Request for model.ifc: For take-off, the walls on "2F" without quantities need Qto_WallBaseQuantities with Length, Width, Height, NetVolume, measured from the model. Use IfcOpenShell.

First a look at what the model holds.

```python
import ifcopenshell
import ifcopenshell.util.element
import ifcopenshell.util.unit

model = ifcopenshell.open("model.ifc")
print(model.schema)
for unit_type in ("LENGTHUNIT", "AREAUNIT", "VOLUMEUNIT"):
    print(unit_type, ifcopenshell.util.unit.calculate_unit_scale(model, unit_type))
storey = next(s for s in model.by_type("IfcBuildingStorey") if s.Name == "2F")
walls = [e for e in ifcopenshell.util.element.get_decomposition(storey) if e.is_a("IfcWall")]
for e in sorted(walls, key=lambda e: e.id()):
    print(e.id(), e.is_a(), e.Name, list(ifcopenshell.util.element.get_psets(e, qtos_only=True)), sep=" | ")
```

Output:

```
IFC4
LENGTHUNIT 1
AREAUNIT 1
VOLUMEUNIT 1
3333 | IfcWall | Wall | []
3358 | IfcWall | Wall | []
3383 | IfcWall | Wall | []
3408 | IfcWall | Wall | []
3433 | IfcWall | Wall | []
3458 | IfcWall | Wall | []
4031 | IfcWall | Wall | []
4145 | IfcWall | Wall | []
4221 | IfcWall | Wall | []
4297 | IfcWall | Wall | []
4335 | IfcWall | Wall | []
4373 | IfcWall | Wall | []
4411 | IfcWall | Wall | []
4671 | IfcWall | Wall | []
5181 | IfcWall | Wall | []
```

```python
import ifcopenshell
import ifcopenshell.api.pset
import ifcopenshell.geom
import ifcopenshell.util.element
import ifcopenshell.util.shape
import ifcopenshell.util.unit

model = ifcopenshell.open("model.ifc")
unit_scale = ifcopenshell.util.unit.calculate_unit_scale(model)
volume_scale = ifcopenshell.util.unit.calculate_unit_scale(model, "VOLUMEUNIT")
settings = ifcopenshell.geom.settings()

storey = next(s for s in model.by_type("IfcBuildingStorey") if s.Name == "2F")
walls = [e for e in ifcopenshell.util.element.get_decomposition(storey) if e.is_a("IfcWall")]

for e in sorted(walls, key=lambda e: e.id()):
    if ifcopenshell.util.element.get_psets(e, qtos_only=True, should_inherit=False):
        continue
    # Geometry comes back in metres, in the element's own axes.
    shape = ifcopenshell.geom.create_shape(settings, e)
    values = {
        "Length": ifcopenshell.util.shape.get_x(shape.geometry) / unit_scale,
        "Width": ifcopenshell.util.shape.get_y(shape.geometry) / unit_scale,
        "Height": ifcopenshell.util.shape.get_z(shape.geometry) / unit_scale,
        "NetVolume": ifcopenshell.util.shape.get_volume(shape.geometry) / volume_scale,
    }
    qto = ifcopenshell.api.pset.add_qto(model, product=e, name="Qto_WallBaseQuantities")
    ifcopenshell.api.pset.edit_qto(model, qto=qto, properties=values)
    print(e.id(), {k: round(v, 3) for k, v in values.items()})

model.write("model-out.ifc")
```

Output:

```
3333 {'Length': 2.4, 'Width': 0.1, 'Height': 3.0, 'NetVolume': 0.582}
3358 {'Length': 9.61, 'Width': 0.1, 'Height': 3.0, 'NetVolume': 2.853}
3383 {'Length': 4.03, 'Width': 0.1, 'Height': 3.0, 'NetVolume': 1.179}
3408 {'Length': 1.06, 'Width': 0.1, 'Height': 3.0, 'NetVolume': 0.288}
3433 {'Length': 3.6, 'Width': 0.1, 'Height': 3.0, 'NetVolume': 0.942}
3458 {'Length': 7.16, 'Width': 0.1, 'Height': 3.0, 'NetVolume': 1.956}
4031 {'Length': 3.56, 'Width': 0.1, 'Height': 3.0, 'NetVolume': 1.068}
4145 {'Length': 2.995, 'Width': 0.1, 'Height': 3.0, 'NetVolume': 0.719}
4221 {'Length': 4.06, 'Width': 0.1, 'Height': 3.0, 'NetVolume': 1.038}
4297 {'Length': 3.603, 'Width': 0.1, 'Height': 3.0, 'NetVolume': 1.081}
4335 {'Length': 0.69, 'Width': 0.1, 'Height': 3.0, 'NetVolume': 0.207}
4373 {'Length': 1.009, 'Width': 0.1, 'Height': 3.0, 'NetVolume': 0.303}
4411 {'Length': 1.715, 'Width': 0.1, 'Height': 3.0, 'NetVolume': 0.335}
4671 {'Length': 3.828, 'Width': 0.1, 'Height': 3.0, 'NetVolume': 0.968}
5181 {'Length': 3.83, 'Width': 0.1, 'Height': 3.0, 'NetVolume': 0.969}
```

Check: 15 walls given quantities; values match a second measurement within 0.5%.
